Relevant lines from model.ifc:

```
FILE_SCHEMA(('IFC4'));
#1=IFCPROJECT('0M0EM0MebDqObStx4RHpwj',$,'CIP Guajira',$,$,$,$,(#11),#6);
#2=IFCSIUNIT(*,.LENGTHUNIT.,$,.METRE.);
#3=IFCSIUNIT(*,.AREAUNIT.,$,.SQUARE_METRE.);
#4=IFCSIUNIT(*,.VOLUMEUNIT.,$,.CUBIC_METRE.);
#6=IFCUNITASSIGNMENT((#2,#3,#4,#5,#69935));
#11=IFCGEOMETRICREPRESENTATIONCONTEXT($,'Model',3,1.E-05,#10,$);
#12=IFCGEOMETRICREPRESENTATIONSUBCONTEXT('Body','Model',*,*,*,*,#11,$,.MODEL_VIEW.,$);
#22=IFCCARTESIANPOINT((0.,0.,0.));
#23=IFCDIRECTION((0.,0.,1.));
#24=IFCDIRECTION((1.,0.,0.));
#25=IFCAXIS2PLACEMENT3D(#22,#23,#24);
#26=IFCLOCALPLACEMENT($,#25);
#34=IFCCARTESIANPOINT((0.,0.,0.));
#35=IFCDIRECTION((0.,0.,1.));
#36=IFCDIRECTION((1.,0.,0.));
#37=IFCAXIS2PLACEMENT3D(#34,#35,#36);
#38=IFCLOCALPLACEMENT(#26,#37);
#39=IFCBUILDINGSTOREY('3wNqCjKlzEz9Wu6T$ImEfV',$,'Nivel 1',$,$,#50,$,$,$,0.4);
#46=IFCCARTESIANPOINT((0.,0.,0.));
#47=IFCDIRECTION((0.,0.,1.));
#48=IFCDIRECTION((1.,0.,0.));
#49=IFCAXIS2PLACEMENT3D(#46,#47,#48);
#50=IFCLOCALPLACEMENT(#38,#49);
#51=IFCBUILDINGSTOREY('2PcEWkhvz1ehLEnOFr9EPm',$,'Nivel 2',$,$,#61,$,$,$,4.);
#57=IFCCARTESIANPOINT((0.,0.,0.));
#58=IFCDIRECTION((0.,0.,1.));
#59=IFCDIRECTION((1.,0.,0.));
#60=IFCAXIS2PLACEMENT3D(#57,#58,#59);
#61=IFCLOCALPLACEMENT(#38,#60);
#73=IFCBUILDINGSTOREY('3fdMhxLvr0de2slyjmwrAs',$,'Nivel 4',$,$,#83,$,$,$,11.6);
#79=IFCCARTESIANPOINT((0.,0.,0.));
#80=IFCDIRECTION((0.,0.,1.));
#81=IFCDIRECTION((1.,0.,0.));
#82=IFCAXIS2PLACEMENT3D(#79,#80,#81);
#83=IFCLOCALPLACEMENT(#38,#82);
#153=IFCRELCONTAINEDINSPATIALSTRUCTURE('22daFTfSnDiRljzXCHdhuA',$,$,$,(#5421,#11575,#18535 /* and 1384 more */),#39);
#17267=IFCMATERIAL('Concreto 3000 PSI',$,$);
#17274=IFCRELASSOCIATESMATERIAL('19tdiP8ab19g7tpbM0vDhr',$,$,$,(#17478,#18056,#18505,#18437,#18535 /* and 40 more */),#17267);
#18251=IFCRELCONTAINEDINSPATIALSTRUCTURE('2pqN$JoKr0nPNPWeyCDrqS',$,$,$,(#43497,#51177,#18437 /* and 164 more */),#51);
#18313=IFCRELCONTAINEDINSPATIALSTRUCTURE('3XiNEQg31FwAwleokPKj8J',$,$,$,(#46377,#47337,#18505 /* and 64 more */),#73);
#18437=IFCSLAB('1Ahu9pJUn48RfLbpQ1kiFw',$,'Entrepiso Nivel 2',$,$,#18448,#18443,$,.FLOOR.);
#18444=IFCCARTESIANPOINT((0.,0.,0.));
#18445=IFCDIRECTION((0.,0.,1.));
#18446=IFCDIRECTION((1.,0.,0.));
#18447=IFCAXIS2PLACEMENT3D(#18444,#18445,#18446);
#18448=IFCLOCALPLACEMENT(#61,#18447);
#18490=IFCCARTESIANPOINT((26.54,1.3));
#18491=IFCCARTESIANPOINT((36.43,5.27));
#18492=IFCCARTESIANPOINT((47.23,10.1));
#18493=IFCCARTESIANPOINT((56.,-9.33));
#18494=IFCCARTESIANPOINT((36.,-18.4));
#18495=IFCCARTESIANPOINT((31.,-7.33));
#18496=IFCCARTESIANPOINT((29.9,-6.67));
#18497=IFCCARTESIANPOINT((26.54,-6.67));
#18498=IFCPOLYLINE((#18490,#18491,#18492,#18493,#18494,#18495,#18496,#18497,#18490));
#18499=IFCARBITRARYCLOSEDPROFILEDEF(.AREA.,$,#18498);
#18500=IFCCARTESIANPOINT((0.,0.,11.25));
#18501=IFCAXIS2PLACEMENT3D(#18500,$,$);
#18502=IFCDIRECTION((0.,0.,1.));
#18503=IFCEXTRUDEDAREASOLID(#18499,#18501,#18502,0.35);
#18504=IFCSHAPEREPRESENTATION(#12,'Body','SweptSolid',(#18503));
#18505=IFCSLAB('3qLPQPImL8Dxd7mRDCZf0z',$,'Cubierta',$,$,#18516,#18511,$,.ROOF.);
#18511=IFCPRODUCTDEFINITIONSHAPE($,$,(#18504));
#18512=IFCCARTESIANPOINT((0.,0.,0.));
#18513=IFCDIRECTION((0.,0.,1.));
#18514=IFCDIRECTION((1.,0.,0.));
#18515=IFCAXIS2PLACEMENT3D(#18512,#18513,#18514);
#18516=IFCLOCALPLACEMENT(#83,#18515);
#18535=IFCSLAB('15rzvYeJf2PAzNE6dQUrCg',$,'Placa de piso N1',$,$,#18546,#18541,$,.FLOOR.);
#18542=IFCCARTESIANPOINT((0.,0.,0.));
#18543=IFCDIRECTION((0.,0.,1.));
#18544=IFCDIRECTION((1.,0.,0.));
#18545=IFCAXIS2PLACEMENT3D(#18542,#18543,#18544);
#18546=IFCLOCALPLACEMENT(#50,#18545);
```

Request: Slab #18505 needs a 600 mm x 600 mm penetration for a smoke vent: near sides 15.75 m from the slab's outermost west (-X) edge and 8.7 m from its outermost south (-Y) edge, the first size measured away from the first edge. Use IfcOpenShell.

```python
import numpy as np
import ifcopenshell
import ifcopenshell.api.feature
import ifcopenshell.api.geometry
import ifcopenshell.api.root
import ifcopenshell.geom
import ifcopenshell.util.placement
import ifcopenshell.util.representation
import ifcopenshell.util.shape
import ifcopenshell.util.unit

model = ifcopenshell.open("model.ifc")
unit_scale = ifcopenshell.util.unit.calculate_unit_scale(model)
settings = ifcopenshell.geom.settings()


def volume(element):
    """Net volume in cubic metres, openings subtracted."""
    shape = ifcopenshell.geom.create_shape(settings, element)
    return ifcopenshell.util.shape.get_volume(shape.geometry)


slab = model.by_id(18505)
before = volume(slab)

# Extent in the slab's own axes, in metres. The edges named are its -X and -Y sides.
slab_shape = ifcopenshell.geom.create_shape(settings, slab)
vertices = ifcopenshell.util.shape.get_vertices(slab_shape.geometry)
x_min, y_min, bottom = vertices.min(axis=0)
top = vertices[:, 2].max()

opening = ifcopenshell.api.root.create_entity(model, ifc_class="IfcOpeningElement", name="Smoke vent opening", predefined_type="OPENING")
context = ifcopenshell.util.representation.get_context(model, "Model", "Body", "MODEL_VIEW")
width, depth = 0.6, 0.6
outline = [(0.0, 0.0), (width, 0.0), (width, depth), (0.0, depth), (0.0, 0.0)]
# Overshoot both faces by 50 mm so the cut is clean.
shape = ifcopenshell.api.geometry.add_slab_representation(
    model, context=context, depth=top - bottom + 0.1, polyline=outline
)
ifcopenshell.api.geometry.assign_representation(model, product=opening, representation=shape)

matrix = ifcopenshell.util.placement.get_local_placement(slab.ObjectPlacement)
matrix[:, 3] = matrix @ np.append(np.array([x_min + 15.75, y_min + 8.7, bottom - 0.05]) / unit_scale, 1.0)
ifcopenshell.api.geometry.edit_object_placement(model, product=opening, matrix=matrix, is_si=False)
ifcopenshell.api.feature.add_feature(model, feature=opening, element=slab)

after = volume(slab)

print(f"slab volume {before:.3f} -> {after:.3f} m3")

model.write("model-out.ifc")
```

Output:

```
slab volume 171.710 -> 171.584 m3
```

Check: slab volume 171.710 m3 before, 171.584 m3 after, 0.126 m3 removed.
